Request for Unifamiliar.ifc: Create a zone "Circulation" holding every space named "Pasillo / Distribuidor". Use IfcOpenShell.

First a look at what the model holds.

```python
import ifcopenshell

model = ifcopenshell.open("Unifamiliar.ifc")
print(model.schema)
seen = {}
for space in model.by_type("IfcSpace"):
    seen[space.LongName] = seen.get(space.LongName, 0) + 1
for name, count in sorted(seen.items(), key=str):
    print(count, "x", name)
print("zones:", [z.Name for z in model.by_type("IfcZone")][:20])
```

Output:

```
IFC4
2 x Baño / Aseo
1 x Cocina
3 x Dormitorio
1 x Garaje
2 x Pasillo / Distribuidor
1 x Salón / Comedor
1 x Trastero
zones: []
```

```python
import ifcopenshell
import ifcopenshell.api.group
import ifcopenshell.api.root

model = ifcopenshell.open("Unifamiliar.ifc")

names = {"Pasillo / Distribuidor"}
spaces = [s for s in model.by_type("IfcSpace") if s.LongName in names]

zone = ifcopenshell.api.root.create_entity(model, ifc_class="IfcZone", name="Circulation")
ifcopenshell.api.group.assign_group(model, products=spaces, group=zone)
print(len(spaces), "spaces in", zone.Name)

model.write("Unifamiliar_v2.ifc")
```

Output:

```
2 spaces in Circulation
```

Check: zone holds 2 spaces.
